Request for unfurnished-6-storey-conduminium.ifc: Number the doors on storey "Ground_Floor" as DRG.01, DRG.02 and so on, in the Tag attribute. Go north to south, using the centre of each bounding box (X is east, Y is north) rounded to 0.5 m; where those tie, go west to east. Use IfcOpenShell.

First a look at what the model holds.

```python
import ifcopenshell
import ifcopenshell.util.element
import ifcopenshell.util.placement

model = ifcopenshell.open("unfurnished-6-storey-conduminium.ifc")
print(model.schema)
storey = next(s for s in model.by_type("IfcBuildingStorey") if s.Name == "Ground_Floor")
doors = [e for e in ifcopenshell.util.element.get_decomposition(storey) if e.is_a("IfcDoor")]
for e in sorted(doors, key=lambda e: e.id()):
    origin = ifcopenshell.util.placement.get_local_placement(e.ObjectPlacement)[:3, 3]
    print(e.id(), e.Tag, e.Name, origin.round(2) + 0.0, sep=" | ")
```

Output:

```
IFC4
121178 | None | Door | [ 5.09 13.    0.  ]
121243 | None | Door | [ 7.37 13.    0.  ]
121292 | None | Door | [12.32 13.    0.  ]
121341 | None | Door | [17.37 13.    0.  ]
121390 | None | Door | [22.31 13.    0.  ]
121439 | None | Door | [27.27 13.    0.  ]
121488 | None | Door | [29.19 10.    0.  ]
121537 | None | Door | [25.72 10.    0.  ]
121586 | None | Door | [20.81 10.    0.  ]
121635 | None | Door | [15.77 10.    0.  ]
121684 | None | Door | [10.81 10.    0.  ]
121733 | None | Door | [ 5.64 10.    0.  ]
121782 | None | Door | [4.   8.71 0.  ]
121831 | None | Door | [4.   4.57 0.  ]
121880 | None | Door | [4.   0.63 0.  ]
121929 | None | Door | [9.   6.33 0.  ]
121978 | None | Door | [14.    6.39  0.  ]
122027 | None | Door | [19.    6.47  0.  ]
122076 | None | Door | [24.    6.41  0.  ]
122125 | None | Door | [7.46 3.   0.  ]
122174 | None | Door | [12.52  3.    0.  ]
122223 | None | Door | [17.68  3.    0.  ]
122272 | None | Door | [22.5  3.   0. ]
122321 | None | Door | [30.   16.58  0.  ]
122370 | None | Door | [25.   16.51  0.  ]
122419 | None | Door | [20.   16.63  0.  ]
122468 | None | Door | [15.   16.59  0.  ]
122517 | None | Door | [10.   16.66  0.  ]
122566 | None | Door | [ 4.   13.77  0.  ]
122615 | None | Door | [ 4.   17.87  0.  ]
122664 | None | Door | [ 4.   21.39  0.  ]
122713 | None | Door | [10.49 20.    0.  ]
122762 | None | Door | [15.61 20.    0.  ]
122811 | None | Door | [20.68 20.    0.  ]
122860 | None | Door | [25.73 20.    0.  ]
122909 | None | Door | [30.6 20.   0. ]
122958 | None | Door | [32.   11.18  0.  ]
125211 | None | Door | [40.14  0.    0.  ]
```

```python
import ifcopenshell
import ifcopenshell.geom
import ifcopenshell.util.element
import ifcopenshell.util.shape

model = ifcopenshell.open("unfurnished-6-storey-conduminium.ifc")
settings = ifcopenshell.geom.settings()
settings.set("use-world-coords", True)


def centre(element):
    shape = ifcopenshell.geom.create_shape(settings, element)
    return ifcopenshell.util.shape.get_bbox_centroid(shape.geometry)


storey = next(s for s in model.by_type("IfcBuildingStorey") if s.Name == "Ground_Floor")
doors = [e for e in ifcopenshell.util.element.get_decomposition(storey) if e.is_a("IfcDoor")]

# Insertion points can sit at a corner or the storey origin, so sort by the geometry (in metres).
centres = {e: centre(e) for e in doors}
doors.sort(key=lambda e: (-round(centres[e][1] / 0.5), centres[e][0]))

for i, e in enumerate(doors, start=1):
    number = f"DRG.{i:02d}"
    e.Tag = number
    print(e.id(), number)

model.write("unfurnished-6-storey-conduminium_updated.ifc")
```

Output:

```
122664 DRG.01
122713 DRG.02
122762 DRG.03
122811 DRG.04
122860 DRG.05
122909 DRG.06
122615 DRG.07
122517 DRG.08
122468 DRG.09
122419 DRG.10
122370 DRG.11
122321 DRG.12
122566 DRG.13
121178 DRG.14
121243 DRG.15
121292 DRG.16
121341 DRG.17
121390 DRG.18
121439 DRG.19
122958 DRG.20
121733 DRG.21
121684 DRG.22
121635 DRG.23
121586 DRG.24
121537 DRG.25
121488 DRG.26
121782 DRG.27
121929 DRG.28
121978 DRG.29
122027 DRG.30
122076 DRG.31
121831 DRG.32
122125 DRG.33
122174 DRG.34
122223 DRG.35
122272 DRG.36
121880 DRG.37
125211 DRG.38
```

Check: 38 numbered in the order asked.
